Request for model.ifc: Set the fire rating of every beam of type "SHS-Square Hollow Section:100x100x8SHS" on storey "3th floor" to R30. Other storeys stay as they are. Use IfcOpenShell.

First a look at what the model holds.

```python
import ifcopenshell
import ifcopenshell.util.element

model = ifcopenshell.open("model.ifc")
print(model.schema)
storey = next(s for s in model.by_type("IfcBuildingStorey") if s.Name == "3th floor")
beams = [e for e in ifcopenshell.util.element.get_decomposition(storey) if e.is_a("IfcBeam")]
seen = {}
for e in beams:
    element_type = ifcopenshell.util.element.get_type(e)
    key = (element_type.Name if element_type != e and element_type else None, ifcopenshell.util.element.get_pset(e, "Pset_BeamCommon", "FireRating"))
    seen[key] = seen.get(key, 0) + 1
for (name, value), count in sorted(seen.items(), key=str):
    print(count, "x", name, "|", value)
```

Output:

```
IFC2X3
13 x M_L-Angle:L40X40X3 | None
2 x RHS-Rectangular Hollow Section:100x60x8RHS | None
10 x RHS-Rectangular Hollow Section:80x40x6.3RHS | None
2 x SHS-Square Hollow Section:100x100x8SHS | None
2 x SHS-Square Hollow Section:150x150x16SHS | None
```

```python
import ifcopenshell
import ifcopenshell.api.pset
import ifcopenshell.util.element

model = ifcopenshell.open("model.ifc")

storey = next(s for s in model.by_type("IfcBuildingStorey") if s.Name == "3th floor")
beams = [e for e in ifcopenshell.util.element.get_decomposition(storey) if e.is_a("IfcBeam")]

count = 0
for e in beams:
    element_type = ifcopenshell.util.element.get_type(e)
    if element_type in (None, e) or element_type.Name != "SHS-Square Hollow Section:100x100x8SHS":
        continue
    # add_pset returns the element's existing set when there is one.
    pset = ifcopenshell.api.pset.add_pset(model, product=e, name="Pset_BeamCommon")
    ifcopenshell.api.pset.edit_pset(model, pset=pset, properties={"FireRating": "R30"})
    count += 1

print(count, "beams updated")

model.write("model_edited.ifc")
```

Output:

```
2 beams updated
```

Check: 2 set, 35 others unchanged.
